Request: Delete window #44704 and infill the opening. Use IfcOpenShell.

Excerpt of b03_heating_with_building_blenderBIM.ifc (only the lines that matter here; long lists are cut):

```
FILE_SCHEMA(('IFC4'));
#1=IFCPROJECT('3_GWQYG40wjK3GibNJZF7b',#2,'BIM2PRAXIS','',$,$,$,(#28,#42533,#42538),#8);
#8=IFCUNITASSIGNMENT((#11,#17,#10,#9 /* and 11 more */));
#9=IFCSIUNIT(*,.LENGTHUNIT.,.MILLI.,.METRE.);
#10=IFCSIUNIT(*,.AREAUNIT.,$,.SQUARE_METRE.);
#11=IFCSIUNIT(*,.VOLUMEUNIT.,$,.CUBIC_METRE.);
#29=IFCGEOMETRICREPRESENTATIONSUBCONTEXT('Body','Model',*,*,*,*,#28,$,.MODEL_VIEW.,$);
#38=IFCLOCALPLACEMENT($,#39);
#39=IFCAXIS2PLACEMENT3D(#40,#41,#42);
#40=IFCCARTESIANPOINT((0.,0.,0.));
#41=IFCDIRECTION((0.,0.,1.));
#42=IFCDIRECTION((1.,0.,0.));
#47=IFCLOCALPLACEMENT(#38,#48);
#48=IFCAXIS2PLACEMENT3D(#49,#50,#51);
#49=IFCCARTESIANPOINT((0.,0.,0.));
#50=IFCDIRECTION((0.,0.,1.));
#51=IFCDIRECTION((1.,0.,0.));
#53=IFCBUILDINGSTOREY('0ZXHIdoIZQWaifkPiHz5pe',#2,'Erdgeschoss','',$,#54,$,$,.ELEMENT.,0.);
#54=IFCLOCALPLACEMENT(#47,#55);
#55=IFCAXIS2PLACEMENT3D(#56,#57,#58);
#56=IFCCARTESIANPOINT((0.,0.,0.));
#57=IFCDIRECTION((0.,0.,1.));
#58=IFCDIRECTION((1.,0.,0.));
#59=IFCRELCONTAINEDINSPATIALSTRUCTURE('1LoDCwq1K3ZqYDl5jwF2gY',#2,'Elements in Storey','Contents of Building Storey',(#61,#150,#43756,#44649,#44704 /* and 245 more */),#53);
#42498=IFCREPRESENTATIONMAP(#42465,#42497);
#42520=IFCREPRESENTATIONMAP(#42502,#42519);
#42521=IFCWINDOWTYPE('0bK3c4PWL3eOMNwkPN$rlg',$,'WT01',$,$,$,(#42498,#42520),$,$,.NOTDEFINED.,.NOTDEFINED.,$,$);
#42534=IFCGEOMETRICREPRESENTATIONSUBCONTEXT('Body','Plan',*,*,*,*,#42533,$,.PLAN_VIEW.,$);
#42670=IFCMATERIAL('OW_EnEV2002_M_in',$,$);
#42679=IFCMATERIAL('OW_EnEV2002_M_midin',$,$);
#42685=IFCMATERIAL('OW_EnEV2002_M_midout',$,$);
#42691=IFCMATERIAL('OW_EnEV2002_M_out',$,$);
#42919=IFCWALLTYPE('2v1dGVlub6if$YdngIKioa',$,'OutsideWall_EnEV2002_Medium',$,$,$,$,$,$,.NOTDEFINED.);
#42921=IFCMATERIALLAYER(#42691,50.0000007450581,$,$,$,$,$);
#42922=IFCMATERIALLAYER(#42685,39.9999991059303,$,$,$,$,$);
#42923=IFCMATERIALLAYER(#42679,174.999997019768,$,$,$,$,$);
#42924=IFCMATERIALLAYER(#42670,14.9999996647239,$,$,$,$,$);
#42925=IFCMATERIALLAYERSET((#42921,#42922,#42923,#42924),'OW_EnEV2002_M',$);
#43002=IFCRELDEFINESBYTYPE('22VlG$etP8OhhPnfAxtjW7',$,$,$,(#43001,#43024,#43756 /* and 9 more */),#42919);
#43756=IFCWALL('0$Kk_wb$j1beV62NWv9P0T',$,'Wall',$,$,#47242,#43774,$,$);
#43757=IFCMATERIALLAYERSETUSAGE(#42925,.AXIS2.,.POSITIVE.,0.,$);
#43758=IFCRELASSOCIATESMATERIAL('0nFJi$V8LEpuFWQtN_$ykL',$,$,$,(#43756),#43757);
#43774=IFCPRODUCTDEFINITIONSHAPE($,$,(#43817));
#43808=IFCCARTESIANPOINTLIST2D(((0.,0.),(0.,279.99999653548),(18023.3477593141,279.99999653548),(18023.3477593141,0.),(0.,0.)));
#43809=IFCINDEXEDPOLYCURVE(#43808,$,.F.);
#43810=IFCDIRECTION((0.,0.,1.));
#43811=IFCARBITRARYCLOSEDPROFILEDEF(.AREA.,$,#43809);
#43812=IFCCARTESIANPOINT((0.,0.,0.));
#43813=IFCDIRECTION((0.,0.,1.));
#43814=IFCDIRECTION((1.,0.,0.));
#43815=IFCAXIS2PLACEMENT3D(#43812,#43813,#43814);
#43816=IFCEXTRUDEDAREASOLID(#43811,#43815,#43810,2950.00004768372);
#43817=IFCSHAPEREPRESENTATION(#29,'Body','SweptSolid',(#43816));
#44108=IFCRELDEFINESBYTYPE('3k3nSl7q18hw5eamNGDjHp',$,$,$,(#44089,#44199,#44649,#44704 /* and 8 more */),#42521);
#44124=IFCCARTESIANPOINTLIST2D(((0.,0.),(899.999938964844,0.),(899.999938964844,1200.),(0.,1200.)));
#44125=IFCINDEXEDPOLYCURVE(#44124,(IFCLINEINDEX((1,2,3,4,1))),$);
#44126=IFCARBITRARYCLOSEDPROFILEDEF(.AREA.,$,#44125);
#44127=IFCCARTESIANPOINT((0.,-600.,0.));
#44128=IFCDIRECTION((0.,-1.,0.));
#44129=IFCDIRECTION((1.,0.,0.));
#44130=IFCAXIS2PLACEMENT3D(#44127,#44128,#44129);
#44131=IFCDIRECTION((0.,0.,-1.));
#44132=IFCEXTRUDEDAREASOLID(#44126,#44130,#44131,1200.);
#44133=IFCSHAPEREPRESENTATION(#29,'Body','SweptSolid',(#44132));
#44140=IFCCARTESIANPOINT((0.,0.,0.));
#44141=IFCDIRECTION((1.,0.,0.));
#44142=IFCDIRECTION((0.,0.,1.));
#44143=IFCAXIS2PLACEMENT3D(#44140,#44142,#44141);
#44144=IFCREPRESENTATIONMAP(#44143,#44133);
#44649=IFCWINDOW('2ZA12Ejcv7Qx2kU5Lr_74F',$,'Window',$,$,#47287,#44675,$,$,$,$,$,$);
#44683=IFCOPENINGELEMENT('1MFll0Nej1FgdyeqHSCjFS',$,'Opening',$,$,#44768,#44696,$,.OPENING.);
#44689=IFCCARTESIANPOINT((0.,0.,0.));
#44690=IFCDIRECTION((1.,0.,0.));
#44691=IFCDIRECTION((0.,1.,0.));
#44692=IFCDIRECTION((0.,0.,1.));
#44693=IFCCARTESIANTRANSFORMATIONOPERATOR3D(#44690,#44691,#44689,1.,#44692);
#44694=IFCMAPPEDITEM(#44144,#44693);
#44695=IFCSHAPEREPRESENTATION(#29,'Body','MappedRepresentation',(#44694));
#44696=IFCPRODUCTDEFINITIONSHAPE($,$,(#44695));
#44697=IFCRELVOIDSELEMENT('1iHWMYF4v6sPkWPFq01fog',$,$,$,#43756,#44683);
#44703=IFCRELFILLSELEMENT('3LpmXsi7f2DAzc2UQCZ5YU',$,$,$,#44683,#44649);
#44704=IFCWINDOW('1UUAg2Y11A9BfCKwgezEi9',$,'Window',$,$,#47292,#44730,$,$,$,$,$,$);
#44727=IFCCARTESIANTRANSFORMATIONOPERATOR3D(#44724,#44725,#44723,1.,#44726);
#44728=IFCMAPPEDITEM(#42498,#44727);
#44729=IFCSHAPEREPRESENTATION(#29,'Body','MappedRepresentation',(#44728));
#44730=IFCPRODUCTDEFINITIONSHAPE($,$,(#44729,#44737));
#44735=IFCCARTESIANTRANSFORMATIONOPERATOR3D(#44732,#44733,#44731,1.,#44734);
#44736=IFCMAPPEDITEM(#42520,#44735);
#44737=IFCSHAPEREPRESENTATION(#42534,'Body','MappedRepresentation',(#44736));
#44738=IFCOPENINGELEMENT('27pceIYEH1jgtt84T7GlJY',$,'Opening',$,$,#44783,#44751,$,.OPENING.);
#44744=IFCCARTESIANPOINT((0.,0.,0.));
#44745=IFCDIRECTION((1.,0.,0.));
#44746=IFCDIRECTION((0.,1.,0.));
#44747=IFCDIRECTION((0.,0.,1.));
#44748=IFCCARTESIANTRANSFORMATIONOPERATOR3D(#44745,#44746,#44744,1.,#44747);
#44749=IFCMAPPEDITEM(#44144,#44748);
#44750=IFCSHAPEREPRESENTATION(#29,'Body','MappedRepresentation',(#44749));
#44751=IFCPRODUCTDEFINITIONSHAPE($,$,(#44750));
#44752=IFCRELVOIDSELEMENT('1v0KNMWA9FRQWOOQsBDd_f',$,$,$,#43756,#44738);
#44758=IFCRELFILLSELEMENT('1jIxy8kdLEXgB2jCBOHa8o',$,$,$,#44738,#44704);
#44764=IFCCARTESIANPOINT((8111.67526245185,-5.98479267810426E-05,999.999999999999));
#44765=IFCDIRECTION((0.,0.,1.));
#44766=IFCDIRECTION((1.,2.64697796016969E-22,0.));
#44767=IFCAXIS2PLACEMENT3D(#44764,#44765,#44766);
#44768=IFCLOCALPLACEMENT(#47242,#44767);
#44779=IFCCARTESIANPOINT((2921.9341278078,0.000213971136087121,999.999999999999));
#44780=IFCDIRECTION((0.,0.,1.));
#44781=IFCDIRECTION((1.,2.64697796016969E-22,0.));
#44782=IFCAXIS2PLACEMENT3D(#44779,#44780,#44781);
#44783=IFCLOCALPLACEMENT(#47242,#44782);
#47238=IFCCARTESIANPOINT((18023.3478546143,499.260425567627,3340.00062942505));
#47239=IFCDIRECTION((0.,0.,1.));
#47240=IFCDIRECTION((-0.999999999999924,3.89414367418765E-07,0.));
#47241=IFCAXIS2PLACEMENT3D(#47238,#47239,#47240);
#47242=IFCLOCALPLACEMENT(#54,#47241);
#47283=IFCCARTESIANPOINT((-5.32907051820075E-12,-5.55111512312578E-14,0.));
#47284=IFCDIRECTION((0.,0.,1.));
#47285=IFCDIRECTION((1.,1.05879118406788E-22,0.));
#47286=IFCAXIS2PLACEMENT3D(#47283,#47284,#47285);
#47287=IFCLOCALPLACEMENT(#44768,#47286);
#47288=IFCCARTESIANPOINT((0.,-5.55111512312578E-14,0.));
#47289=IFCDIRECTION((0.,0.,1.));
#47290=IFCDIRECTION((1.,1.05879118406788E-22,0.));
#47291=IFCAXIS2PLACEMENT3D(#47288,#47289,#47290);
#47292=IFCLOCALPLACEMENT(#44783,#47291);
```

```python
import ifcopenshell
import ifcopenshell.api.feature
import ifcopenshell.api.root
import ifcopenshell.geom
import ifcopenshell.util.shape

model = ifcopenshell.open("b03_heating_with_building_blenderBIM.ifc")
settings = ifcopenshell.geom.settings()


def volume(element):
    """Net volume in cubic metres, openings subtracted."""
    shape = ifcopenshell.geom.create_shape(settings, element)
    return ifcopenshell.util.shape.get_volume(shape.geometry)


window = model.by_guid("1UUAg2Y11A9BfCKwgezEi9")
opening = window.FillsVoids[0].RelatingOpeningElement
wall = opening.VoidsElements[0].RelatingBuildingElement
before = volume(wall)

ifcopenshell.api.root.remove_product(model, product=window)
ifcopenshell.api.feature.remove_feature(model, feature=opening)

after = volume(wall)

print(f"wall volume {before:.3f} -> {after:.3f} m3")

model.write("b03_heating_with_building_blenderBIM_rev.ifc")
```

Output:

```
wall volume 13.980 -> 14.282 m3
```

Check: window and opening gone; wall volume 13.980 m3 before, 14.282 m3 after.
